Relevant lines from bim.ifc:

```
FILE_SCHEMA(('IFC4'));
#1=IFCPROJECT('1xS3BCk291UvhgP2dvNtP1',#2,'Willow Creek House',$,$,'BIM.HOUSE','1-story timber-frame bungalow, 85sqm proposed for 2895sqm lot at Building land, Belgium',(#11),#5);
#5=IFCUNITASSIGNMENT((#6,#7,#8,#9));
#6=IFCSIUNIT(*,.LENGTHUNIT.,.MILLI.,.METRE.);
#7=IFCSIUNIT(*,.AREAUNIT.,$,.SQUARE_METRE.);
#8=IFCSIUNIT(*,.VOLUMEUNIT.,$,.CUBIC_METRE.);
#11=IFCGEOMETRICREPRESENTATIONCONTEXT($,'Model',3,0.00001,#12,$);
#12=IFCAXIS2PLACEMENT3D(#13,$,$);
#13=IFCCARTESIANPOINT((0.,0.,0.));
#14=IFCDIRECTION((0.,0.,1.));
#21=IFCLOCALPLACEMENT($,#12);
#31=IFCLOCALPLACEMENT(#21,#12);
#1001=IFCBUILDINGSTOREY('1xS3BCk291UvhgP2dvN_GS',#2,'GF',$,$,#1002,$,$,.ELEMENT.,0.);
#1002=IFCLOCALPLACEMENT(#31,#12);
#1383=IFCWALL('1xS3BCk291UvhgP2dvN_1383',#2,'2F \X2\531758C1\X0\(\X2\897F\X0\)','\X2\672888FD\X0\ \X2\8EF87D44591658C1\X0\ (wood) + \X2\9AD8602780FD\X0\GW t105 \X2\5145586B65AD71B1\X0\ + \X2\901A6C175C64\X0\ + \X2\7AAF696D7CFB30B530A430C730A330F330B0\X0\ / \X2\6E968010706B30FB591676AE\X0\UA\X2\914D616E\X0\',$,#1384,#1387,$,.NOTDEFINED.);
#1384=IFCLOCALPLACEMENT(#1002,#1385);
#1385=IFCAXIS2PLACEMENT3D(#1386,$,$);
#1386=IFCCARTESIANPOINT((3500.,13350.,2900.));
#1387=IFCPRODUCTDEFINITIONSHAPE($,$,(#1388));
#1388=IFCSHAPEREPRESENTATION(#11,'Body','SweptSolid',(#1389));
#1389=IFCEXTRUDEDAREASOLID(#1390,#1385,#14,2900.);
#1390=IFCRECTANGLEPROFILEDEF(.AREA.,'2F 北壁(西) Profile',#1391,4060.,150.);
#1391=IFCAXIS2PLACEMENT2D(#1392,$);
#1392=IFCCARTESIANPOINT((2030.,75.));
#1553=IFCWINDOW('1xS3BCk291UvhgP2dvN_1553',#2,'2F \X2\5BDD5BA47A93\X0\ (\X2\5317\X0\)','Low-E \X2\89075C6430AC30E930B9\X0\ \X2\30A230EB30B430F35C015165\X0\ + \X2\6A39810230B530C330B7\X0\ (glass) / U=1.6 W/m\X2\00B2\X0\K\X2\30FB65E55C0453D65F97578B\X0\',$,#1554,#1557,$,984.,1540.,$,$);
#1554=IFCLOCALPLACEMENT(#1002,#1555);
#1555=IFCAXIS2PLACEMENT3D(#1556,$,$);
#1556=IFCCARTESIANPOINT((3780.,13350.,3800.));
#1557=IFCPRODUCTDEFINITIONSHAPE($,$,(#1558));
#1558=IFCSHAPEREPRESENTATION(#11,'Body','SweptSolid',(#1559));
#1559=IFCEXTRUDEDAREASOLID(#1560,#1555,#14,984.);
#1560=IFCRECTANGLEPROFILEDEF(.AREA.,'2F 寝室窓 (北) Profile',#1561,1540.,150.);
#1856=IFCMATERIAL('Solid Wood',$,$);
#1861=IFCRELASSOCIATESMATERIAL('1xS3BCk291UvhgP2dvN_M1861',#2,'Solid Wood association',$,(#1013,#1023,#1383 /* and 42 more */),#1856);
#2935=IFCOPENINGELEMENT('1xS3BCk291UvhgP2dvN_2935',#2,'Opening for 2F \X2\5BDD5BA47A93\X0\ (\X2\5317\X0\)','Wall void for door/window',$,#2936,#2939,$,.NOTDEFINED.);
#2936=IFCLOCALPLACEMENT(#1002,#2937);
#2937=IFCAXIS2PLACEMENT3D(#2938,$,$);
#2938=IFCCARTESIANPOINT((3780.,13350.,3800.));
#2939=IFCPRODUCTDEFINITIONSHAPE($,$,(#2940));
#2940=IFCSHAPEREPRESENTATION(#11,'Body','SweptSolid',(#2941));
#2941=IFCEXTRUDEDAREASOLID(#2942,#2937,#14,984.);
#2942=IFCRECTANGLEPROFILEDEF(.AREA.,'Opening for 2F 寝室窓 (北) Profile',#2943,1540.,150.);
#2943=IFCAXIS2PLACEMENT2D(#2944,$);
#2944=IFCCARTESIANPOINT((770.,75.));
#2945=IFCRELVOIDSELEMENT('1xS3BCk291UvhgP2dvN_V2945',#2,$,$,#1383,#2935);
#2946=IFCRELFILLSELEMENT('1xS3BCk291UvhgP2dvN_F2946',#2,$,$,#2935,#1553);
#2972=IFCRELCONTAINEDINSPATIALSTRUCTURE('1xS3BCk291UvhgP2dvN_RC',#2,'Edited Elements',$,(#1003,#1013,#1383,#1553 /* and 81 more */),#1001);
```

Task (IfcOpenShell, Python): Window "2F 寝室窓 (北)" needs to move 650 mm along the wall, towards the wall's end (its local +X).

```python
import ifcopenshell
import ifcopenshell.api.geometry
import ifcopenshell.util.placement
import ifcopenshell.util.unit

model = ifcopenshell.open("bim.ifc")
unit_scale = ifcopenshell.util.unit.calculate_unit_scale(model)

window = model.by_guid("1xS3BCk291UvhgP2dvN_1553")
opening = window.FillsVoids[0].RelatingOpeningElement
wall = opening.VoidsElements[0].RelatingBuildingElement

wall_matrix = ifcopenshell.util.placement.get_local_placement(wall.ObjectPlacement)
shift = wall_matrix[:3, 0] * 0.65 / unit_scale
before = ifcopenshell.util.placement.get_local_placement(window.ObjectPlacement)[:3, 3].copy()

# The window is not placed relative to its opening, so move both.
for product in (opening, window):
    matrix = ifcopenshell.util.placement.get_local_placement(product.ObjectPlacement)
    matrix[:3, 3] += shift
    ifcopenshell.api.geometry.edit_object_placement(model, product=product, matrix=matrix, is_si=False)

after = ifcopenshell.util.placement.get_local_placement(window.ObjectPlacement)[:3, 3]
print("window moved by", (after - before).round(3) + 0.0)

model.write("bim_updated.ifc")
```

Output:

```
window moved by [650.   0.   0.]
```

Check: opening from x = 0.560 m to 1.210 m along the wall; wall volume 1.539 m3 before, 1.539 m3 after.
